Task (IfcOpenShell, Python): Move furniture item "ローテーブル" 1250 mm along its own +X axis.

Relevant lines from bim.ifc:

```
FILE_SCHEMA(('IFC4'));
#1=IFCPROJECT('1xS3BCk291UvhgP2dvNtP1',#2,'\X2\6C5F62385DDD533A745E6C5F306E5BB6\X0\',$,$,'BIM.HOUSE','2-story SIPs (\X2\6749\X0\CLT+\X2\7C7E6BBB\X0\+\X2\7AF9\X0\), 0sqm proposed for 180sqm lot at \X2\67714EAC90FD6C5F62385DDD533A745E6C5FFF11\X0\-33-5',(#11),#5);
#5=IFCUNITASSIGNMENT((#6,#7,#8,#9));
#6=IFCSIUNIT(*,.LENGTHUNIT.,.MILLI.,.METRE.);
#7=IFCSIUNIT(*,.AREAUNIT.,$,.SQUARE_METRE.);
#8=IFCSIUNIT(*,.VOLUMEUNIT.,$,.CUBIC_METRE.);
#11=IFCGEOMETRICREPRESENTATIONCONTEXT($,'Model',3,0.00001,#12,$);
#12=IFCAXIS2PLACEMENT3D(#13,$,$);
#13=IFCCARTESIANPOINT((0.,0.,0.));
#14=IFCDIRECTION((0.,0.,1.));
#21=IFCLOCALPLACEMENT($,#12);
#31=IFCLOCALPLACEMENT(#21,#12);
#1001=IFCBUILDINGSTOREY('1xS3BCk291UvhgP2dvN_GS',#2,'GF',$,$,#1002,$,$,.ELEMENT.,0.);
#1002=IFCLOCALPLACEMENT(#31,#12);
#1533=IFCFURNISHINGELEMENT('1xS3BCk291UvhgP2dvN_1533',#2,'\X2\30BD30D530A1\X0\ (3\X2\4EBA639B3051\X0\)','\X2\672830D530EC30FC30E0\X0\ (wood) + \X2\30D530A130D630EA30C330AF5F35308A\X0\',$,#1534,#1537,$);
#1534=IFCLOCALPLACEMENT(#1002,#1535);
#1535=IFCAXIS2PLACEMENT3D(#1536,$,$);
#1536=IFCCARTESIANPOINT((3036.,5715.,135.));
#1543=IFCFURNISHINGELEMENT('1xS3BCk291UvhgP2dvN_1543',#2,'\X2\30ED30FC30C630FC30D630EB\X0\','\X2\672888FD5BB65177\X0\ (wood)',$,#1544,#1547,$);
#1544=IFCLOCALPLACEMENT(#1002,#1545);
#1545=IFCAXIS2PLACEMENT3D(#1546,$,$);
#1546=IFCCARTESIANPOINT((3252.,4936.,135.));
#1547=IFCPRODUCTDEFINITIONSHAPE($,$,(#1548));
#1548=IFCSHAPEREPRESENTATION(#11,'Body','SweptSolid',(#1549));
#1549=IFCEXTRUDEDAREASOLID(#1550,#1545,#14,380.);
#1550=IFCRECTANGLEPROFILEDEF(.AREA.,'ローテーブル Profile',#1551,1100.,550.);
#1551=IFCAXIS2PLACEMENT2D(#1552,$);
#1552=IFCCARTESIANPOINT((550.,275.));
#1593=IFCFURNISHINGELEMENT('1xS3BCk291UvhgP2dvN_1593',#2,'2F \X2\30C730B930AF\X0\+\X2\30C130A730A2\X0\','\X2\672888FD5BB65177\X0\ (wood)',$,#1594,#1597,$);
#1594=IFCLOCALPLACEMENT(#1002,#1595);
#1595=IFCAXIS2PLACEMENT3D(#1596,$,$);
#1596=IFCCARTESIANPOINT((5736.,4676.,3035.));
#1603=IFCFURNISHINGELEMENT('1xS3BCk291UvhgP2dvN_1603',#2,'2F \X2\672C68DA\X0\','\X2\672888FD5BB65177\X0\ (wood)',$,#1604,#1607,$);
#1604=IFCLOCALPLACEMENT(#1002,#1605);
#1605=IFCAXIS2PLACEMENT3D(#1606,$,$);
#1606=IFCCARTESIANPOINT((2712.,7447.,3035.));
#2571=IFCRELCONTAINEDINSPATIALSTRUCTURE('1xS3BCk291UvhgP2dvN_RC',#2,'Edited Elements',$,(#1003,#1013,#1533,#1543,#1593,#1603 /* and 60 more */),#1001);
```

```python
import ifcopenshell
import ifcopenshell.api.geometry
import ifcopenshell.util.placement

model = ifcopenshell.open("bim.ifc")

item = model.by_guid("1xS3BCk291UvhgP2dvN_1543")
matrix = ifcopenshell.util.placement.get_local_placement(item.ObjectPlacement)
matrix[:3, 3] += matrix[:3, 0] * 1250.0
ifcopenshell.api.geometry.edit_object_placement(model, product=item, matrix=matrix, is_si=False)

print(ifcopenshell.util.placement.get_local_placement(item.ObjectPlacement).round(3) + 0.0)

model.write("bim_rev.ifc")
```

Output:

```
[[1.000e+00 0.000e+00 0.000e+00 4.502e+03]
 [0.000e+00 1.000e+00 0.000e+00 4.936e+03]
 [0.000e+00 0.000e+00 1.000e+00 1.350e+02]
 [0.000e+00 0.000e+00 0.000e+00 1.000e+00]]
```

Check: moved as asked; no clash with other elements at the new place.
